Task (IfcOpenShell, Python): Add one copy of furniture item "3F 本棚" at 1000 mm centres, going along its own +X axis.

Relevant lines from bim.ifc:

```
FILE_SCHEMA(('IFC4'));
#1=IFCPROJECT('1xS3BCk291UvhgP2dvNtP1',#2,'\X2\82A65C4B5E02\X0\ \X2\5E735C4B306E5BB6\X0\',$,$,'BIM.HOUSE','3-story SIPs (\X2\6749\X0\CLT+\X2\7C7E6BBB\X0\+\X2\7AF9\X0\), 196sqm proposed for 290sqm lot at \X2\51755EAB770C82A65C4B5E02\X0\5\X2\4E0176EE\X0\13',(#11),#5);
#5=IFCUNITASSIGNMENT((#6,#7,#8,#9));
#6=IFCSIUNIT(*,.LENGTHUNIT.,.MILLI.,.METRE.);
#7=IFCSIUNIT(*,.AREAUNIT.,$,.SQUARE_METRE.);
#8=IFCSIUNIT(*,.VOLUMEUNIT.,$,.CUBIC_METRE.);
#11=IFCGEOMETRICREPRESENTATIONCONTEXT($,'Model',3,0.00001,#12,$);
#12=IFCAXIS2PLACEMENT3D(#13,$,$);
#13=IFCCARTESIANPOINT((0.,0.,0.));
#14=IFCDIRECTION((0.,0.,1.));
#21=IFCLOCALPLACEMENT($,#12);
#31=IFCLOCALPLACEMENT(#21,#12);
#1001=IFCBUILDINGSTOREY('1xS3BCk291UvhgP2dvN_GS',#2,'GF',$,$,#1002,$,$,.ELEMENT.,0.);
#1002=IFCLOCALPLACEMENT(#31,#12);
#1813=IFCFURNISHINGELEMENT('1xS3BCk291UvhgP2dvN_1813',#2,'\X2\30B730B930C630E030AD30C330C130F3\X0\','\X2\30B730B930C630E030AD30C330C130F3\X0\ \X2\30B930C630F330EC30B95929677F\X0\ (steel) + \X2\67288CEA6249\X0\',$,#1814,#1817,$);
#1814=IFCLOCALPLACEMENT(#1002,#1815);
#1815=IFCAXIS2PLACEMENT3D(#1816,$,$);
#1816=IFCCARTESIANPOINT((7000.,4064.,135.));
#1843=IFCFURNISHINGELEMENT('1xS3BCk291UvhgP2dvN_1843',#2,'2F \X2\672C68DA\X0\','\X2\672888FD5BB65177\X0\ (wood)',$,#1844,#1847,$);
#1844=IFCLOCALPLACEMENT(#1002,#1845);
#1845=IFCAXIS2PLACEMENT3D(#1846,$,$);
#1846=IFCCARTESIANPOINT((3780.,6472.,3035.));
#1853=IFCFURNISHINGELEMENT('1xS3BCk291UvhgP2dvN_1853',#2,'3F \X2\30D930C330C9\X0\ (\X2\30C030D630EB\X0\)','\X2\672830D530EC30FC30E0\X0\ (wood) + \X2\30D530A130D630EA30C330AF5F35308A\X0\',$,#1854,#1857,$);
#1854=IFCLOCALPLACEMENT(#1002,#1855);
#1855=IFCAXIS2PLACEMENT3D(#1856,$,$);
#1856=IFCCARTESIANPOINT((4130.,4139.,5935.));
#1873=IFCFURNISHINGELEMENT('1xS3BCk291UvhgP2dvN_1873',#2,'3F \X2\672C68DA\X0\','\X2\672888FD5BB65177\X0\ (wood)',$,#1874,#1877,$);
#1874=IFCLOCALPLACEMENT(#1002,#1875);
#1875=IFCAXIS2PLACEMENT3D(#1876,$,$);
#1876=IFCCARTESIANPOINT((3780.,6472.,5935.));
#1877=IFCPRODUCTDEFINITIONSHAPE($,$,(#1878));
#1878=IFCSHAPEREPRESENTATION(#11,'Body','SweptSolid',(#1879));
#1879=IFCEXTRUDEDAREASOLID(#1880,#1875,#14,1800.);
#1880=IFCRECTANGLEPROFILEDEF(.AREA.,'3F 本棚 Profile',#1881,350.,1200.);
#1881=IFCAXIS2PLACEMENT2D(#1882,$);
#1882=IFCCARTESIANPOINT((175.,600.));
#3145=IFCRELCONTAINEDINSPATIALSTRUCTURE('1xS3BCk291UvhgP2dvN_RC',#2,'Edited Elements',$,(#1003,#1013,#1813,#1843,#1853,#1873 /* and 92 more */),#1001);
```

```python
import ifcopenshell
import ifcopenshell.api.geometry
import ifcopenshell.api.root
import ifcopenshell.util.element
import ifcopenshell.util.placement
import ifcopenshell.util.unit

model = ifcopenshell.open("bim.ifc")
unit_scale = ifcopenshell.util.unit.calculate_unit_scale(model)


def reuse_history(source, copy):
    """copy_class also copies each property set's owner history, people and application; keep the originals."""
    for rel in copy.IsDefinedBy:
        if rel.is_a("IfcRelDefinesByProperties") and (history := rel.RelatingPropertyDefinition.OwnerHistory):
            rel.RelatingPropertyDefinition.OwnerHistory = source.OwnerHistory
            ifcopenshell.util.element.remove_deep2(model, history)


source = model.by_guid("1xS3BCk291UvhgP2dvN_1873")
base = ifcopenshell.util.placement.get_local_placement(source.ObjectPlacement)
step = base[:3, 0] * 1 / unit_scale

for i in range(1, 2):
    copy = ifcopenshell.api.root.copy_class(model, product=source)
    copy.Representation = ifcopenshell.util.element.copy_deep(
        model, source.Representation, exclude=["IfcGeometricRepresentationContext", "IfcRepresentationMap"]
    )
    reuse_history(source, copy)
    matrix = base.copy()
    matrix[:3, 3] += i * step
    print("added at", matrix[:3, 3].round(3) + 0.0)
    ifcopenshell.api.geometry.edit_object_placement(model, product=copy, matrix=matrix, is_si=False)

model.write("bim_v2.ifc")
```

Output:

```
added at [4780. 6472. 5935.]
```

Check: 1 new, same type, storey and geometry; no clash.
